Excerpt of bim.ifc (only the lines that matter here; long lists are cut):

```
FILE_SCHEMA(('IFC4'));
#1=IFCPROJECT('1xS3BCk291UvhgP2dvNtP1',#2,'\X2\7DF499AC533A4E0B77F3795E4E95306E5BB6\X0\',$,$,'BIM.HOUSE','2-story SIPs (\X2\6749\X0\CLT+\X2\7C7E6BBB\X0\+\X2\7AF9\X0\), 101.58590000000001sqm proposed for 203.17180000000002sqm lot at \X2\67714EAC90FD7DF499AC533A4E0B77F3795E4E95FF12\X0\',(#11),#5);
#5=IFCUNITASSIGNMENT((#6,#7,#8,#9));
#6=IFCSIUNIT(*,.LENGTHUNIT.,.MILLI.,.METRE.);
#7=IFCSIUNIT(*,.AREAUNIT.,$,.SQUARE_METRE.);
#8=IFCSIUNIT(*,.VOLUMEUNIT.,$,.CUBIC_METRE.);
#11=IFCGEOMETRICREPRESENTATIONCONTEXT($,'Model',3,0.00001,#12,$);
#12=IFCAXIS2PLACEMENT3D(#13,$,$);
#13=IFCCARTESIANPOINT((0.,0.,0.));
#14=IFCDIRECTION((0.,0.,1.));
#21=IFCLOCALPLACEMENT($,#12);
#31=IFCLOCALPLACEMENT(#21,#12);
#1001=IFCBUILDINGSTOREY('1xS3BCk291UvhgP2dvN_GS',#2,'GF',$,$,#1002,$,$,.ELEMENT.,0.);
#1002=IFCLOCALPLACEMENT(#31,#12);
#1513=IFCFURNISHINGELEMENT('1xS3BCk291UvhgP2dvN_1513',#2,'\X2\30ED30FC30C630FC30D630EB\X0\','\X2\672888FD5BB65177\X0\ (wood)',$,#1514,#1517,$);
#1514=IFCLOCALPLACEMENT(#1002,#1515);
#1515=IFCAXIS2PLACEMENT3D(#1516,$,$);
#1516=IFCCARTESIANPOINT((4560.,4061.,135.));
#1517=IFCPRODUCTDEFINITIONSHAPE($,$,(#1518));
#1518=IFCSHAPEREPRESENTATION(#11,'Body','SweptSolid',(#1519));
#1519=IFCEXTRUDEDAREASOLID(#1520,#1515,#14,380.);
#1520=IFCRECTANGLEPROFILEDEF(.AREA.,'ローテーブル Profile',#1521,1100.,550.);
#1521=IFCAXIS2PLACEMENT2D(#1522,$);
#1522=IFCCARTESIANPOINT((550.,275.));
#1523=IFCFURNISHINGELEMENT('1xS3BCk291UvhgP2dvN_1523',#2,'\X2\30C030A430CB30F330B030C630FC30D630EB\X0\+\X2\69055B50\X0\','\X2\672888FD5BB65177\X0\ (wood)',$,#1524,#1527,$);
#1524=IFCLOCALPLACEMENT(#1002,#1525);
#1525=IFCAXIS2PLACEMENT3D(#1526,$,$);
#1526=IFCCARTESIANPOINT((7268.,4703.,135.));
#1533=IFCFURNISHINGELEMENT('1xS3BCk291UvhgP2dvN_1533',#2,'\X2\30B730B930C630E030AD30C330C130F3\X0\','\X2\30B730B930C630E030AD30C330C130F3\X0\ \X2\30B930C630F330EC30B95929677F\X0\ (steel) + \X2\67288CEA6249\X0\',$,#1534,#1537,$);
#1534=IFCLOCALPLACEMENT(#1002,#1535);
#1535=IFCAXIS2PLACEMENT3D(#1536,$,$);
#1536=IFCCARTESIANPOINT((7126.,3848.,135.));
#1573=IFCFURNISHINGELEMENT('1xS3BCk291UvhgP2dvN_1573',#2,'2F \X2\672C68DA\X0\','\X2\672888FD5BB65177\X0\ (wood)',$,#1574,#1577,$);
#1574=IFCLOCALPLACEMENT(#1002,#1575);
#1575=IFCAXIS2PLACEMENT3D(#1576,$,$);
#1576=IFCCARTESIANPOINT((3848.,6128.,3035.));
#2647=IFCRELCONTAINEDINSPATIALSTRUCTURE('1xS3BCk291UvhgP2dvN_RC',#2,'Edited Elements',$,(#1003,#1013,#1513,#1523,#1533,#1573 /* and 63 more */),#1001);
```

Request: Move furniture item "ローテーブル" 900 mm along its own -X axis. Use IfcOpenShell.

```python
import ifcopenshell
import ifcopenshell.api.geometry
import ifcopenshell.util.placement
import ifcopenshell.util.unit

model = ifcopenshell.open("bim.ifc")
unit_scale = ifcopenshell.util.unit.calculate_unit_scale(model)

item = model.by_guid("1xS3BCk291UvhgP2dvN_1513")
matrix = ifcopenshell.util.placement.get_local_placement(item.ObjectPlacement)
matrix[:3, 3] -= matrix[:3, 0] * 0.9 / unit_scale
ifcopenshell.api.geometry.edit_object_placement(model, product=item, matrix=matrix, is_si=False)

print(ifcopenshell.util.placement.get_local_placement(item.ObjectPlacement).round(3) + 0.0)

model.write("bim_v2.ifc")
```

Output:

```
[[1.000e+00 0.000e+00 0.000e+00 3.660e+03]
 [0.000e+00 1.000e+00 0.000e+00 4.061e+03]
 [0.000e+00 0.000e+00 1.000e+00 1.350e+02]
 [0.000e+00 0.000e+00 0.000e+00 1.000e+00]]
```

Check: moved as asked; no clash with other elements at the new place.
